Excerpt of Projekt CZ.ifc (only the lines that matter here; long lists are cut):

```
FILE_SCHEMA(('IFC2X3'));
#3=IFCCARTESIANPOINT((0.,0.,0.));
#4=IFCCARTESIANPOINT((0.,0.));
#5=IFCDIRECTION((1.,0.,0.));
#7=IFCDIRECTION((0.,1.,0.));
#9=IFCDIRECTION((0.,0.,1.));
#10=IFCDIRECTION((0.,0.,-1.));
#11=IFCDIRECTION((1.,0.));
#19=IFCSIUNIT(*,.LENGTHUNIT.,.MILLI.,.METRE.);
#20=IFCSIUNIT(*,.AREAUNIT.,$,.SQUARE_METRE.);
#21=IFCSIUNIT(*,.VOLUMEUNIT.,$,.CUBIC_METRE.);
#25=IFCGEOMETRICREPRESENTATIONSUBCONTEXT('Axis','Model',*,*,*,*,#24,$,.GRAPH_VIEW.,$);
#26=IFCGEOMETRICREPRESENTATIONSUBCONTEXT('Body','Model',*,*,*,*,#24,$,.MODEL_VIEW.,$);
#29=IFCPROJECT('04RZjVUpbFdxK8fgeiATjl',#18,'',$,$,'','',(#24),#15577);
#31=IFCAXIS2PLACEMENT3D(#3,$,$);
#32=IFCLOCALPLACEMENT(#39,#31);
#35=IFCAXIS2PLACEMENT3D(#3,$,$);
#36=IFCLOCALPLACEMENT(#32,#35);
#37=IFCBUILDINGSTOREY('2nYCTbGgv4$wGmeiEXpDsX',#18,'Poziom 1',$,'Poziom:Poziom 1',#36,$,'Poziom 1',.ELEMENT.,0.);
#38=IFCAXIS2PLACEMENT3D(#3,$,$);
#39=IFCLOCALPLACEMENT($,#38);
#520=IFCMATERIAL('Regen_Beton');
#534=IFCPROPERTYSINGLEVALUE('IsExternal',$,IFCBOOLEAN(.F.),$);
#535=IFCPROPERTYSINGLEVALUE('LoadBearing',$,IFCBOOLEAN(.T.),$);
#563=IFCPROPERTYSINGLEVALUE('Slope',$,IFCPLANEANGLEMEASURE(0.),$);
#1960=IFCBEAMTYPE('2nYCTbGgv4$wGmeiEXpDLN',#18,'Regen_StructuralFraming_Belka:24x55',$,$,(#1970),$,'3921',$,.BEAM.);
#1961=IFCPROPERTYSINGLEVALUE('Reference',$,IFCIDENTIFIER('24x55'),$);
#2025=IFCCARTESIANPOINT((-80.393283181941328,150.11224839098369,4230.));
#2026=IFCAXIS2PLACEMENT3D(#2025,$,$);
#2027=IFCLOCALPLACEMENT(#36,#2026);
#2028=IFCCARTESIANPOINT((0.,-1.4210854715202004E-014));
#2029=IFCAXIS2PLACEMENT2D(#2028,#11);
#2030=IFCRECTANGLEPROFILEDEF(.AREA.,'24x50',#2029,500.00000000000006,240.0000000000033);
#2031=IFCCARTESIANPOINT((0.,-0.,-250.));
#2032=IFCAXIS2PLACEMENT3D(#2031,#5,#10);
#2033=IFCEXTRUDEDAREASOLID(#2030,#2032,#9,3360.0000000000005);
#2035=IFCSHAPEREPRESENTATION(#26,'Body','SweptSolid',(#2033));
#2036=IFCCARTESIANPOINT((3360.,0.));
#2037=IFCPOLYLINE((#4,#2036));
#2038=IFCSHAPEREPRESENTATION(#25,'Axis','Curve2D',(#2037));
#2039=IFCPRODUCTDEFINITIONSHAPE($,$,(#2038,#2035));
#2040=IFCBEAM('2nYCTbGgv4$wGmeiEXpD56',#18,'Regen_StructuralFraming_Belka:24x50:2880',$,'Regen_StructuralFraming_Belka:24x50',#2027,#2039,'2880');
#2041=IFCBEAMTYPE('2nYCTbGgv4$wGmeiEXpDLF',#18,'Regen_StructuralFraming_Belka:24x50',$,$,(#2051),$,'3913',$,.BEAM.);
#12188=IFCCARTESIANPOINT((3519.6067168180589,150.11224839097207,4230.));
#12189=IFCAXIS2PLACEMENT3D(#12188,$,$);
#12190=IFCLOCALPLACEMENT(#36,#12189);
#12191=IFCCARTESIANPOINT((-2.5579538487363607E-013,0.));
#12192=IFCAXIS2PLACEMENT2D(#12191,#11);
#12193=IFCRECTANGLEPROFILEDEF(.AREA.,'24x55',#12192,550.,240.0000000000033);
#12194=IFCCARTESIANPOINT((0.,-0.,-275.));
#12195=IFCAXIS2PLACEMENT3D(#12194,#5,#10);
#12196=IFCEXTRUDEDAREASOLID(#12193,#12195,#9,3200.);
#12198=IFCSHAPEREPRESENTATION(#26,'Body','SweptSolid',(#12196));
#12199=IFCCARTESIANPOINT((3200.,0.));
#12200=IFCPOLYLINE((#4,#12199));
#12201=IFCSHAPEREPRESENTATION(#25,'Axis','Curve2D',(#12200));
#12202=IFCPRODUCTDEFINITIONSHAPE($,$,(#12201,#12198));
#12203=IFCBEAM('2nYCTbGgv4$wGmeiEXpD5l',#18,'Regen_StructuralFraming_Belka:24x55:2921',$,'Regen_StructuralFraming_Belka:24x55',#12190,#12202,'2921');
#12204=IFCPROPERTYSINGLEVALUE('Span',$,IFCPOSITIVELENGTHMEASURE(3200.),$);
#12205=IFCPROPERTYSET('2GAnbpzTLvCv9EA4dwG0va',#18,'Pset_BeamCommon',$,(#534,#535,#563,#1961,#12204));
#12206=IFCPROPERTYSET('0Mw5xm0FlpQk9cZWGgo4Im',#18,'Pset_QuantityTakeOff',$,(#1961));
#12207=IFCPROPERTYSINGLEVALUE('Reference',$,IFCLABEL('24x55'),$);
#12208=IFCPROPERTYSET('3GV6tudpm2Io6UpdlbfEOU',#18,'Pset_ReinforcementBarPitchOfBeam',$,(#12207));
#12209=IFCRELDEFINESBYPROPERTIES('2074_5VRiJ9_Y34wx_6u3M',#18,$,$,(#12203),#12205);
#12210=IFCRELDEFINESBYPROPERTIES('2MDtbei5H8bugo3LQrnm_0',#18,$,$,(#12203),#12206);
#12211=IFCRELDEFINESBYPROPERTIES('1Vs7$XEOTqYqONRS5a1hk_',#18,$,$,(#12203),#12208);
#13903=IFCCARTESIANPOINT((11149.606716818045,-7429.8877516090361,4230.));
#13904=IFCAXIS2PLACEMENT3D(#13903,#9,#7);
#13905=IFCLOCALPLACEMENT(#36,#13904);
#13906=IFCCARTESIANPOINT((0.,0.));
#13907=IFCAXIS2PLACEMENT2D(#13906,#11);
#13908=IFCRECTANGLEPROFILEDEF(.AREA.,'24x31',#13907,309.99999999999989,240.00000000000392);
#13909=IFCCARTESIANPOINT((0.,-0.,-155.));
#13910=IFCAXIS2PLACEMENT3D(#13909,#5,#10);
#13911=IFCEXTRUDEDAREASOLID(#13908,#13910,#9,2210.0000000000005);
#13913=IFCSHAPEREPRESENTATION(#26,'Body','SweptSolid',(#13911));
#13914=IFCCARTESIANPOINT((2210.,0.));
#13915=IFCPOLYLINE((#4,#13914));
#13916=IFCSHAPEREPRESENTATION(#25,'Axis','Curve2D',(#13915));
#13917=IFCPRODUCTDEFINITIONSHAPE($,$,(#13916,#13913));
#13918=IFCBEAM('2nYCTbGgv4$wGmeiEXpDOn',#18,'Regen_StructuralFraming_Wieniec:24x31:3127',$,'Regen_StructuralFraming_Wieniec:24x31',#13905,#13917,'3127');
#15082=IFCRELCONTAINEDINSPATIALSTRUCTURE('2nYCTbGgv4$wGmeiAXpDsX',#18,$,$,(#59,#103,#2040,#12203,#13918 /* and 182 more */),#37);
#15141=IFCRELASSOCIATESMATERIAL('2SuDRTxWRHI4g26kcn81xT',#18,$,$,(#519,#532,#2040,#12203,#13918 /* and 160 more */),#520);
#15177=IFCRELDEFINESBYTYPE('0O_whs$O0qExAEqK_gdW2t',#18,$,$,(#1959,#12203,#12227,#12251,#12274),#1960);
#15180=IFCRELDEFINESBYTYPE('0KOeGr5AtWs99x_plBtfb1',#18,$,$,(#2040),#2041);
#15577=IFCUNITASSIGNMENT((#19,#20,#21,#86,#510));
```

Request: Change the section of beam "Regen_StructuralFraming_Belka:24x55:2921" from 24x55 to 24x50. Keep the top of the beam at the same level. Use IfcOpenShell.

```python
import ifcopenshell
import ifcopenshell.api.pset
import ifcopenshell.api.type
import ifcopenshell.util.element
import ifcopenshell.util.representation

model = ifcopenshell.open("Projekt CZ.ifc")

member = model.by_guid("2nYCTbGgv4$wGmeiEXpD5l")
source = next(p for p in model.by_type("IfcRectangleProfileDef") if p.ProfileName == "24x50")

body = ifcopenshell.util.representation.get_representation(member, "Model", "Body")
solid = body.Items[0]
old_profile = solid.SweptArea

# Copy the section's sizes but keep this member's own profile position.
profile = ifcopenshell.util.element.copy(model, source)
# Profiles are centred, so shift by half the change in depth to hold the top.
shift = (old_profile.XDim - profile.XDim) / 2
x, y = old_profile.Position.Location.Coordinates
up = (-1.0, 0.0)  # upwards, in the solid's own plane
location = model.createIfcCartesianPoint((x + up[0] * shift, y + up[1] * shift))
profile.Position = model.createIfcAxis2Placement2D(location, old_profile.Position.RefDirection)
solid.SweptArea = profile
if not model.get_total_inverses(old_profile):
    ifcopenshell.util.element.remove_deep2(model, old_profile)

new_type = model.by_guid("2nYCTbGgv4$wGmeiEXpDLF")
ifcopenshell.api.type.assign_type(
    model, related_objects=[member], relating_type=new_type, should_map_representations=False
)
member.Name = member.Name.replace("24x55", "24x50")
member.ObjectType = "Regen_StructuralFraming_Belka:24x50"
pset = model.by_id(ifcopenshell.util.element.get_pset(member, "Pset_BeamCommon", should_inherit=False)["id"])
ifcopenshell.api.pset.edit_pset(model, pset=pset, properties={"Reference": "24x50"})
pset = model.by_id(ifcopenshell.util.element.get_pset(member, "Pset_QuantityTakeOff", should_inherit=False)["id"])
ifcopenshell.api.pset.edit_pset(model, pset=pset, properties={"Reference": "24x50"})
pset = model.by_id(ifcopenshell.util.element.get_pset(member, "Pset_ReinforcementBarPitchOfBeam", should_inherit=False)["id"])
ifcopenshell.api.pset.edit_pset(model, pset=pset, properties={"Reference": "24x50"})

print(solid.SweptArea)

model.write("Projekt CZ_rev.ifc")
```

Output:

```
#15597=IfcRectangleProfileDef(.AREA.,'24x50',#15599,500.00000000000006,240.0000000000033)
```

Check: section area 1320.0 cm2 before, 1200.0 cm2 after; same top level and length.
